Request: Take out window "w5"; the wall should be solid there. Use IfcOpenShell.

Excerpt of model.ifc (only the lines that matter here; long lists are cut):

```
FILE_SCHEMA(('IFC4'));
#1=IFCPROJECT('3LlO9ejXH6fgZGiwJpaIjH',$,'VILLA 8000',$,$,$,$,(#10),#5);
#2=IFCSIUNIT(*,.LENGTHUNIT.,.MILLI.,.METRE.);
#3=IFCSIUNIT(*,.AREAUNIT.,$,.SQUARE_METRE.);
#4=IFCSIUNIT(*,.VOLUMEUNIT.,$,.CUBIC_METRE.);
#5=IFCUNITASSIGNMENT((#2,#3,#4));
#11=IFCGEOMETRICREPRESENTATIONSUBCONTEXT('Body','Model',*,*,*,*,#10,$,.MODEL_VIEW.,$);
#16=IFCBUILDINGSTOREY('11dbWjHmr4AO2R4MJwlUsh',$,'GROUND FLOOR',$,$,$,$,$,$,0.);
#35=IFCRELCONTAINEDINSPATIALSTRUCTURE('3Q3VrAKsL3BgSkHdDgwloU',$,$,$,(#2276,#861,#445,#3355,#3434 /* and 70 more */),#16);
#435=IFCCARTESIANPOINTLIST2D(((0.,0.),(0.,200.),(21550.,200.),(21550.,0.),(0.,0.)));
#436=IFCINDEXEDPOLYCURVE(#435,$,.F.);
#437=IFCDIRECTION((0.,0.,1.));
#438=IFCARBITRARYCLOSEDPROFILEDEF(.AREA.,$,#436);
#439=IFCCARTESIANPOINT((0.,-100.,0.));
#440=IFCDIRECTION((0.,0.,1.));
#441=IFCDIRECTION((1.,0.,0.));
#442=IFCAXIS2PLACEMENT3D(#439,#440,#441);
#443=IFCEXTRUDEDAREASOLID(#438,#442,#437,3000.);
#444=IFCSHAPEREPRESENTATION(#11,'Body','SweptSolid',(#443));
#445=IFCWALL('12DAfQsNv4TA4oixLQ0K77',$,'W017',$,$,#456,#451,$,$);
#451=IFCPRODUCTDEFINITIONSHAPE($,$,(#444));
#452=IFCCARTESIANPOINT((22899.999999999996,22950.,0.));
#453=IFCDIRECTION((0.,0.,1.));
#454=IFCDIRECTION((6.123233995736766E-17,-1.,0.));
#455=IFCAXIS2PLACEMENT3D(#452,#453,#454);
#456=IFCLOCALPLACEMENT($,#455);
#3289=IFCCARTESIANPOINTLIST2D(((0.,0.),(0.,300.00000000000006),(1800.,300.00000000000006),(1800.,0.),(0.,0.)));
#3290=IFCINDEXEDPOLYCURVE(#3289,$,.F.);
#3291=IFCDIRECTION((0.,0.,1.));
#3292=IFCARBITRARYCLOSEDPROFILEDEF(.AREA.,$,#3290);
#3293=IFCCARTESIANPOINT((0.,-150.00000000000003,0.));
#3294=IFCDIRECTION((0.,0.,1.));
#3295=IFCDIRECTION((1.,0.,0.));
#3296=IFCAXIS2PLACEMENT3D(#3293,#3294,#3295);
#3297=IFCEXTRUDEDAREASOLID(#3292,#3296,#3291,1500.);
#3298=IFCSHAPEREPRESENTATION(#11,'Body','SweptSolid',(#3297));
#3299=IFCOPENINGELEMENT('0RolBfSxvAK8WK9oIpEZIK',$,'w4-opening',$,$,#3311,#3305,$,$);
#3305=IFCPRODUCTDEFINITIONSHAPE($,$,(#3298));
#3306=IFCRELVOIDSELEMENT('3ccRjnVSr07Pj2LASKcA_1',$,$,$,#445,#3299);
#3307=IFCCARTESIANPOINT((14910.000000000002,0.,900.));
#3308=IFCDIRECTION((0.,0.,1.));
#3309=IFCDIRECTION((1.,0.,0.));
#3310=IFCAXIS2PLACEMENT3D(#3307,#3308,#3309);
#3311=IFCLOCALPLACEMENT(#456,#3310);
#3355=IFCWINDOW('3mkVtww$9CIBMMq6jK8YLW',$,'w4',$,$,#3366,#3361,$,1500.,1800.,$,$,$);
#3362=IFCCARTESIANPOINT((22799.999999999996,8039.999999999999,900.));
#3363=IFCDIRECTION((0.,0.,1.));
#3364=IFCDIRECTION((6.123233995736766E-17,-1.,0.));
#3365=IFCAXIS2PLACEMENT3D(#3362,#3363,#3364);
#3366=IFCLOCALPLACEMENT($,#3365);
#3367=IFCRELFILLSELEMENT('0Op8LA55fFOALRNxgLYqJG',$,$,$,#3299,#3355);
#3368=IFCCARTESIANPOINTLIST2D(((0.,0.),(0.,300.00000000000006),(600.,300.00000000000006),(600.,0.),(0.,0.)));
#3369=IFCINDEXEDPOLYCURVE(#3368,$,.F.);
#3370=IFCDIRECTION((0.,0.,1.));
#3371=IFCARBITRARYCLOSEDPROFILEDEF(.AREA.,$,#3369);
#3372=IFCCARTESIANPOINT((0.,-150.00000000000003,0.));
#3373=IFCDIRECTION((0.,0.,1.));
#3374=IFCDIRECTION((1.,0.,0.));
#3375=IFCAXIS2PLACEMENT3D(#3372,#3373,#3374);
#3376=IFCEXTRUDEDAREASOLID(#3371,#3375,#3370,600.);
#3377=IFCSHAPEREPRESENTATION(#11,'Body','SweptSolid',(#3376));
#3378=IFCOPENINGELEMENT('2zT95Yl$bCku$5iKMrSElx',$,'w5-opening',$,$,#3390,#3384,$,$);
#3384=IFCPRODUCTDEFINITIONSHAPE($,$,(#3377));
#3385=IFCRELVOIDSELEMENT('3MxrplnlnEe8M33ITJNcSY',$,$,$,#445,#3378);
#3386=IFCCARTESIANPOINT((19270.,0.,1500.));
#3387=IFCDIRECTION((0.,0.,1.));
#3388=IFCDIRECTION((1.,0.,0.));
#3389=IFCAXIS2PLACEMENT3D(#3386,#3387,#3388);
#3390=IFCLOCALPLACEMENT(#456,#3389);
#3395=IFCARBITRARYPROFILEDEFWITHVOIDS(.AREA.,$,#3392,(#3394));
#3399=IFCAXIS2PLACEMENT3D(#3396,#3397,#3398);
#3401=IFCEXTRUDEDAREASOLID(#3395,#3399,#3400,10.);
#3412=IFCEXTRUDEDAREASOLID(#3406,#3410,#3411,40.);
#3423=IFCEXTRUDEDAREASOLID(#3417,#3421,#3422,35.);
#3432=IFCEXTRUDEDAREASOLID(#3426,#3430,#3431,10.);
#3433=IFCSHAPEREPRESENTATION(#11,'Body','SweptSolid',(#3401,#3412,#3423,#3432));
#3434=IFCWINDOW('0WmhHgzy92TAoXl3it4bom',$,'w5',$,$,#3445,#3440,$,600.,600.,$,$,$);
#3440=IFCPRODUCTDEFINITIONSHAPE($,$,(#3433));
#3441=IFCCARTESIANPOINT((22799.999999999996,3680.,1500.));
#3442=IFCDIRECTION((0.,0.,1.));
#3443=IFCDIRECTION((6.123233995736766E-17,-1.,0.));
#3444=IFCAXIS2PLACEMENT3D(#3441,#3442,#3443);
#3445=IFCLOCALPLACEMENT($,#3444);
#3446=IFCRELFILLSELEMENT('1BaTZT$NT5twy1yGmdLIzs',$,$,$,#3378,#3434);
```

```python
import ifcopenshell
import ifcopenshell.api.feature
import ifcopenshell.api.root
import ifcopenshell.geom
import ifcopenshell.util.shape

model = ifcopenshell.open("model.ifc")
settings = ifcopenshell.geom.settings()


def volume(element):
    """Net volume in cubic metres, openings subtracted."""
    shape = ifcopenshell.geom.create_shape(settings, element)
    return ifcopenshell.util.shape.get_volume(shape.geometry)


window = model.by_guid("0WmhHgzy92TAoXl3it4bom")
opening = window.FillsVoids[0].RelatingOpeningElement
wall = opening.VoidsElements[0].RelatingBuildingElement
before = volume(wall)

ifcopenshell.api.root.remove_product(model, product=window)
ifcopenshell.api.feature.remove_feature(model, feature=opening)

after = volume(wall)

print(f"wall volume {before:.3f} -> {after:.3f} m3")

model.write("model_v2.ifc")
```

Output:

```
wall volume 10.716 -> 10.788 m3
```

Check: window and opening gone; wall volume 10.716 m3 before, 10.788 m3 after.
